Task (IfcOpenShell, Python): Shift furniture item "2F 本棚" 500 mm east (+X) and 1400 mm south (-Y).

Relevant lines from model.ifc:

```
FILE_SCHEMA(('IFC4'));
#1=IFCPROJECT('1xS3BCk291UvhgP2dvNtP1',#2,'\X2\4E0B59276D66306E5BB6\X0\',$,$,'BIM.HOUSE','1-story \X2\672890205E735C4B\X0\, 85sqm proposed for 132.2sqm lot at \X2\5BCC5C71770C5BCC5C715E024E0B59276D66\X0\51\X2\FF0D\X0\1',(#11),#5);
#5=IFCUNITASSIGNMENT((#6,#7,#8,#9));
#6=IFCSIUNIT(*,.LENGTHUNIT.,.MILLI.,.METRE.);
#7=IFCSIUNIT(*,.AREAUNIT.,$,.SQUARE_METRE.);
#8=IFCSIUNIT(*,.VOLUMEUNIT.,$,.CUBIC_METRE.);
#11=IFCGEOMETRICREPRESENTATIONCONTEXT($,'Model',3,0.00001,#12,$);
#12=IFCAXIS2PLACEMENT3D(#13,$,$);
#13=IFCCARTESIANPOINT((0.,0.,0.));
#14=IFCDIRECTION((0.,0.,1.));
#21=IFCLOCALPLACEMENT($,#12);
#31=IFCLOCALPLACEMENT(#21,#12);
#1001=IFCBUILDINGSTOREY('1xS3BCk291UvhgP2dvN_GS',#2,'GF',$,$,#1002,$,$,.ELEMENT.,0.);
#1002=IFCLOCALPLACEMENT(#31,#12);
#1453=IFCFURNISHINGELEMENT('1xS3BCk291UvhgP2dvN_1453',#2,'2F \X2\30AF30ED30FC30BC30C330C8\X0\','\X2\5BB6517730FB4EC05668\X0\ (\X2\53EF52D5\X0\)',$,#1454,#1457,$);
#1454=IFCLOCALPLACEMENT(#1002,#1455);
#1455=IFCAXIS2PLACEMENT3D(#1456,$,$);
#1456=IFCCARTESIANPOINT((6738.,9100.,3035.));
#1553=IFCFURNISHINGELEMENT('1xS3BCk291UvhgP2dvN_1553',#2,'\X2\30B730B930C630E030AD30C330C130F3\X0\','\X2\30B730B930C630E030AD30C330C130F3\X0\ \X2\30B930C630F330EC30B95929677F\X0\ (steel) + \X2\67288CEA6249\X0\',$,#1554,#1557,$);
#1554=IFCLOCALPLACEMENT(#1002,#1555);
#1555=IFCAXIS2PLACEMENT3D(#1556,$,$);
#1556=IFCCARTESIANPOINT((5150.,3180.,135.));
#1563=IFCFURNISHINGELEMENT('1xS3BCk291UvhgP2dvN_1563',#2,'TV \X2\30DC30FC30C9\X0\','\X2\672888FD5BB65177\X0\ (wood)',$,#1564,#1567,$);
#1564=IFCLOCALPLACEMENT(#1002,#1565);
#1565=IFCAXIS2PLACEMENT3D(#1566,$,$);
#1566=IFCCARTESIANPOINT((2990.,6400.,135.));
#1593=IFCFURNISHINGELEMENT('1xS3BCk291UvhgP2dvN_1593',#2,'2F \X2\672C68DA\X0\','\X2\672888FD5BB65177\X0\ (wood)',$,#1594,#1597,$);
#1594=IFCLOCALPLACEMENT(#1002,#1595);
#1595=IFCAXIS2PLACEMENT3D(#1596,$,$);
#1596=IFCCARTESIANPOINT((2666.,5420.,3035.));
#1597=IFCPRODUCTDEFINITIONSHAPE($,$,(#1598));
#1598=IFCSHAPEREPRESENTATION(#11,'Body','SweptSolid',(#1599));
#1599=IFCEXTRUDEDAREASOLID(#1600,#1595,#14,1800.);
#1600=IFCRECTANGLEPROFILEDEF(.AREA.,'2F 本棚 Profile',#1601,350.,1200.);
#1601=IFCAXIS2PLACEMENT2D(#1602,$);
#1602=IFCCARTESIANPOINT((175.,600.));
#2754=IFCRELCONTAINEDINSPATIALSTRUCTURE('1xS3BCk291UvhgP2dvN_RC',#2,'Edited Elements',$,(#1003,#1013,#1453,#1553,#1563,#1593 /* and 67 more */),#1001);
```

```python
import ifcopenshell
import ifcopenshell.api.geometry
import ifcopenshell.util.placement
import ifcopenshell.util.unit

model = ifcopenshell.open("model.ifc")
unit_scale = ifcopenshell.util.unit.calculate_unit_scale(model)

item = model.by_guid("1xS3BCk291UvhgP2dvN_1593")
matrix = ifcopenshell.util.placement.get_local_placement(item.ObjectPlacement)
matrix[0, 3] += 0.5 / unit_scale
matrix[1, 3] -= 1.4 / unit_scale
ifcopenshell.api.geometry.edit_object_placement(model, product=item, matrix=matrix, is_si=False)

print(ifcopenshell.util.placement.get_local_placement(item.ObjectPlacement).round(3) + 0.0)

model.write("model_v2.ifc")
```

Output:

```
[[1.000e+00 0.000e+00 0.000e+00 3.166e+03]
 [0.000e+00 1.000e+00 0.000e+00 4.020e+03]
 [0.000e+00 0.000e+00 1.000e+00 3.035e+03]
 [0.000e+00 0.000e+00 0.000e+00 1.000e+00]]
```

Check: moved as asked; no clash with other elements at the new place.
